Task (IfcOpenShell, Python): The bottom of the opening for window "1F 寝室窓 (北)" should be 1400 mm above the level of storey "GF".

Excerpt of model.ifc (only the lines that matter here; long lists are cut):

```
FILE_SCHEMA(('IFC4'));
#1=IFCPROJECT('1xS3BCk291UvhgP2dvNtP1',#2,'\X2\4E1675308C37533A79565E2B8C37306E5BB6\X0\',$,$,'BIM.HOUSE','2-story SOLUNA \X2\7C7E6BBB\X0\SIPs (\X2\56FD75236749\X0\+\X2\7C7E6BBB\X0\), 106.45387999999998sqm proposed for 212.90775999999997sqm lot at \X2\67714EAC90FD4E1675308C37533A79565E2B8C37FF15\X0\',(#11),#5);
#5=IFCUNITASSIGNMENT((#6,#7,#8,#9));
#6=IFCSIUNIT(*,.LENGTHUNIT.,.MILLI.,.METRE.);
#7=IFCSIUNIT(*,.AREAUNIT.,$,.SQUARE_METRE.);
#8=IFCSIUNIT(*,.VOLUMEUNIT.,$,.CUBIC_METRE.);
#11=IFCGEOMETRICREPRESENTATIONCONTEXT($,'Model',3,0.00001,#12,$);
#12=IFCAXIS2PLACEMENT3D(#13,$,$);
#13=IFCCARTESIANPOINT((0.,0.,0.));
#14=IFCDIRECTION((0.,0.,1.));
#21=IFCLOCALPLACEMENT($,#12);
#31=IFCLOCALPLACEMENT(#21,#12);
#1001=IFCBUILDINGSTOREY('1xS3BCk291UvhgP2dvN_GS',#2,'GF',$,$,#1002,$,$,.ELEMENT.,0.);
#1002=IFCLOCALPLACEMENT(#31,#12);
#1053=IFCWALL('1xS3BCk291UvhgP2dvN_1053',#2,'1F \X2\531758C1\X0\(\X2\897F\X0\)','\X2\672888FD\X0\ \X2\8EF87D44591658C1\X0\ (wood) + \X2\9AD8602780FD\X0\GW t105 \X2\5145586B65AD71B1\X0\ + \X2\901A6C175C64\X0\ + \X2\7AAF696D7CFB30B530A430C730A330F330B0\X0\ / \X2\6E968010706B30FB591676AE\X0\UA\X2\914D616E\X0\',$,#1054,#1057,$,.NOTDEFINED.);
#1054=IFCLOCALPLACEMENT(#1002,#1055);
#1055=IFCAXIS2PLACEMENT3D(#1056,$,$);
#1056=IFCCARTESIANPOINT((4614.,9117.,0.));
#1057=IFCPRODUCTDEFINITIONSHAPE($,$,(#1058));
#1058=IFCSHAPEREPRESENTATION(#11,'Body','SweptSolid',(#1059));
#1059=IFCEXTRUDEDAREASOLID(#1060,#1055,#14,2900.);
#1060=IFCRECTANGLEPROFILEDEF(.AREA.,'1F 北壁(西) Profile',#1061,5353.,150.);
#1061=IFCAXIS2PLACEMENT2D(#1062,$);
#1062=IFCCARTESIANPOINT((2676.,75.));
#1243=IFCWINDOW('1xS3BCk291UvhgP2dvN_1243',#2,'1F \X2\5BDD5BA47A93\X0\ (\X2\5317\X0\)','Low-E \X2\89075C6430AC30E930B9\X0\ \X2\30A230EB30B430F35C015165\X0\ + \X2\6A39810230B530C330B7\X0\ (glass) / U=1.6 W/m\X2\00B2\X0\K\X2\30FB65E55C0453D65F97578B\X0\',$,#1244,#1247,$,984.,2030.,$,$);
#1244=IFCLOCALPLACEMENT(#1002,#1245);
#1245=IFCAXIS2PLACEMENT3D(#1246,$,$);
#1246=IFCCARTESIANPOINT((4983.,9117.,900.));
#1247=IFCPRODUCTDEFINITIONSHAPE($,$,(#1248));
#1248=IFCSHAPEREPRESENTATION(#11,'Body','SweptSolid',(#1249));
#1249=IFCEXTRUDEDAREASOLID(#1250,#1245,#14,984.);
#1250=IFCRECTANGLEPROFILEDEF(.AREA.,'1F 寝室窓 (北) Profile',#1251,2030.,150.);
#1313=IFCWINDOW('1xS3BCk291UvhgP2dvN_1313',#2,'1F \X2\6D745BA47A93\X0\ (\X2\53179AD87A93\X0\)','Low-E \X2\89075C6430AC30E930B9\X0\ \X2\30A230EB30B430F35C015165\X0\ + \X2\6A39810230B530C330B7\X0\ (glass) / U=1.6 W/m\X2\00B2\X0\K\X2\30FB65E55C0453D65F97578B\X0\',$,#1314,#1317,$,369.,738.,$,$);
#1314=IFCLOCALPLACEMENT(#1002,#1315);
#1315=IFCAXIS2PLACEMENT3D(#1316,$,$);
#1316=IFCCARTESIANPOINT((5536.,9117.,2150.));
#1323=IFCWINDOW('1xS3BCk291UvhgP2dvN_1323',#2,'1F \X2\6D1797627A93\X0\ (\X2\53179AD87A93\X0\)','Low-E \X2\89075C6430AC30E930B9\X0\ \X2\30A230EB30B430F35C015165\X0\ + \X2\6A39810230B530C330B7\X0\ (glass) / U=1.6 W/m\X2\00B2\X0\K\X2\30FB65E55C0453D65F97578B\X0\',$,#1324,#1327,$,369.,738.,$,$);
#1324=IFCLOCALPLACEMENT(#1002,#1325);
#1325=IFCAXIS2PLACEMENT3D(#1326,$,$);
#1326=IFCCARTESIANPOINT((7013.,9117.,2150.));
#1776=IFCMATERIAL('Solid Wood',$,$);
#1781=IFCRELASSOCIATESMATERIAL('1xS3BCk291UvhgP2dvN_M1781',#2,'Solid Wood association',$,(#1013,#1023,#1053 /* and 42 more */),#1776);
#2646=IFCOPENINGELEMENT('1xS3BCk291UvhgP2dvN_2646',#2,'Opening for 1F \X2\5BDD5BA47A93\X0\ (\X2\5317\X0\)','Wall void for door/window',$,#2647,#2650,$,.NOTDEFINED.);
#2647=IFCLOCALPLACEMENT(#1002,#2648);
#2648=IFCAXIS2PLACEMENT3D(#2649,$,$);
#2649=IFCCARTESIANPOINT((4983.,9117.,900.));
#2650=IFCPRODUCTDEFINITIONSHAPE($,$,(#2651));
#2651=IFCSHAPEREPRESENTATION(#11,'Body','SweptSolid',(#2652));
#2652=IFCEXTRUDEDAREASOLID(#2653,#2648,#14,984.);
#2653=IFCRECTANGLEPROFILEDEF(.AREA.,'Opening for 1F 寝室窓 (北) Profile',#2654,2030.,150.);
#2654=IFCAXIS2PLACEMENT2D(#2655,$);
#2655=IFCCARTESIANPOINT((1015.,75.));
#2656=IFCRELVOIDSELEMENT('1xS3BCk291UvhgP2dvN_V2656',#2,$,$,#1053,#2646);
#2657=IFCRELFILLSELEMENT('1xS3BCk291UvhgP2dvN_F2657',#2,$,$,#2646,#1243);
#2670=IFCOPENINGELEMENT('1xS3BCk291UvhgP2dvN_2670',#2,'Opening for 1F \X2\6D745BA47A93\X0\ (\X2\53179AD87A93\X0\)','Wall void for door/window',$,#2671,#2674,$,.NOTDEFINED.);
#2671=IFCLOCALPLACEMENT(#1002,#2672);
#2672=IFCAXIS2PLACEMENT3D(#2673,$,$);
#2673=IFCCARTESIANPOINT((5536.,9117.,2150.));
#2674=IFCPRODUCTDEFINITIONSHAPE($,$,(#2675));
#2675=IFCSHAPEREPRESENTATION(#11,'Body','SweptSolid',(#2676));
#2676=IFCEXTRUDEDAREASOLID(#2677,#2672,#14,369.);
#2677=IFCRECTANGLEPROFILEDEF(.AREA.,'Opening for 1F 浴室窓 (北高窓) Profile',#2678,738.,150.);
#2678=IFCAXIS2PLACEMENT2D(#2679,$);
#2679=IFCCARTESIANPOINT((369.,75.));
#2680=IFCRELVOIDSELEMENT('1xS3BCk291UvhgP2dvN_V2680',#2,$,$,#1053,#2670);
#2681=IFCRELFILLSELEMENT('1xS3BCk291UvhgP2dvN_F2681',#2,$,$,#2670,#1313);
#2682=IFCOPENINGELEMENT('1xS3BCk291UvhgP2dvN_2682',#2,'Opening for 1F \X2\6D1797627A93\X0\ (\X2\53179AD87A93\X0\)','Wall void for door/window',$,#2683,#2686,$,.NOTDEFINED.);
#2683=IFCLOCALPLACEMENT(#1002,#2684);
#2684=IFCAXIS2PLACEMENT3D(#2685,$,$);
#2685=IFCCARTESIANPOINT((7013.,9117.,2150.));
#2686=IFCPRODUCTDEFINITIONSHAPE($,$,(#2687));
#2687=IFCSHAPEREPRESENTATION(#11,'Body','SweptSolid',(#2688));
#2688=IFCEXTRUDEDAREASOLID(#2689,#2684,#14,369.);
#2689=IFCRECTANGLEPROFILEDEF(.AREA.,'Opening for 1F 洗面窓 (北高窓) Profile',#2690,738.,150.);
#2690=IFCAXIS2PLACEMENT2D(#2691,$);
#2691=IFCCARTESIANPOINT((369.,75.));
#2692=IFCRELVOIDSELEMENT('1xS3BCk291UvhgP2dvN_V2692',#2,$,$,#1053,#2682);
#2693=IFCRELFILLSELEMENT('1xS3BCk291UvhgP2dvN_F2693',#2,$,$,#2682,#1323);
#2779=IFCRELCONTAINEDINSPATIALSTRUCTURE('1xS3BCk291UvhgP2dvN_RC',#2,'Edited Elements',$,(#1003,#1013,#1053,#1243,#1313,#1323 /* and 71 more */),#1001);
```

```python
import numpy as np
import ifcopenshell
import ifcopenshell.api.geometry
import ifcopenshell.geom
import ifcopenshell.util.element
import ifcopenshell.util.placement
import ifcopenshell.util.shape
import ifcopenshell.util.unit

model = ifcopenshell.open("model.ifc")
unit_scale = ifcopenshell.util.unit.calculate_unit_scale(model)

window = model.by_guid("1xS3BCk291UvhgP2dvN_1243")
opening = window.FillsVoids[0].RelatingOpeningElement
storey = ifcopenshell.util.element.get_container(window, ifc_class="IfcBuildingStorey")
level = ifcopenshell.util.placement.get_local_placement(storey.ObjectPlacement)[2, 3]

# The opening's origin need not be at the sill, so measure its lowest point.
shape = ifcopenshell.geom.create_shape(ifcopenshell.geom.settings(), opening)
bottom = ifcopenshell.util.shape.get_shape_bottom_elevation(shape, shape.geometry) / unit_scale
dz = level + 1.4 / unit_scale - bottom

shift = np.array([0.0, 0.0, dz])
# The window is not placed relative to its opening, so move both.
for product in (opening, window):
    matrix = ifcopenshell.util.placement.get_local_placement(product.ObjectPlacement)
    matrix[:3, 3] += shift
    ifcopenshell.api.geometry.edit_object_placement(model, product=product, matrix=matrix, is_si=False)

print(f"moved by {dz * unit_scale:+.3f} m")

model.write("model_updated.ifc")
```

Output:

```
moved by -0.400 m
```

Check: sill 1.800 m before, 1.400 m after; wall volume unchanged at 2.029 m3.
